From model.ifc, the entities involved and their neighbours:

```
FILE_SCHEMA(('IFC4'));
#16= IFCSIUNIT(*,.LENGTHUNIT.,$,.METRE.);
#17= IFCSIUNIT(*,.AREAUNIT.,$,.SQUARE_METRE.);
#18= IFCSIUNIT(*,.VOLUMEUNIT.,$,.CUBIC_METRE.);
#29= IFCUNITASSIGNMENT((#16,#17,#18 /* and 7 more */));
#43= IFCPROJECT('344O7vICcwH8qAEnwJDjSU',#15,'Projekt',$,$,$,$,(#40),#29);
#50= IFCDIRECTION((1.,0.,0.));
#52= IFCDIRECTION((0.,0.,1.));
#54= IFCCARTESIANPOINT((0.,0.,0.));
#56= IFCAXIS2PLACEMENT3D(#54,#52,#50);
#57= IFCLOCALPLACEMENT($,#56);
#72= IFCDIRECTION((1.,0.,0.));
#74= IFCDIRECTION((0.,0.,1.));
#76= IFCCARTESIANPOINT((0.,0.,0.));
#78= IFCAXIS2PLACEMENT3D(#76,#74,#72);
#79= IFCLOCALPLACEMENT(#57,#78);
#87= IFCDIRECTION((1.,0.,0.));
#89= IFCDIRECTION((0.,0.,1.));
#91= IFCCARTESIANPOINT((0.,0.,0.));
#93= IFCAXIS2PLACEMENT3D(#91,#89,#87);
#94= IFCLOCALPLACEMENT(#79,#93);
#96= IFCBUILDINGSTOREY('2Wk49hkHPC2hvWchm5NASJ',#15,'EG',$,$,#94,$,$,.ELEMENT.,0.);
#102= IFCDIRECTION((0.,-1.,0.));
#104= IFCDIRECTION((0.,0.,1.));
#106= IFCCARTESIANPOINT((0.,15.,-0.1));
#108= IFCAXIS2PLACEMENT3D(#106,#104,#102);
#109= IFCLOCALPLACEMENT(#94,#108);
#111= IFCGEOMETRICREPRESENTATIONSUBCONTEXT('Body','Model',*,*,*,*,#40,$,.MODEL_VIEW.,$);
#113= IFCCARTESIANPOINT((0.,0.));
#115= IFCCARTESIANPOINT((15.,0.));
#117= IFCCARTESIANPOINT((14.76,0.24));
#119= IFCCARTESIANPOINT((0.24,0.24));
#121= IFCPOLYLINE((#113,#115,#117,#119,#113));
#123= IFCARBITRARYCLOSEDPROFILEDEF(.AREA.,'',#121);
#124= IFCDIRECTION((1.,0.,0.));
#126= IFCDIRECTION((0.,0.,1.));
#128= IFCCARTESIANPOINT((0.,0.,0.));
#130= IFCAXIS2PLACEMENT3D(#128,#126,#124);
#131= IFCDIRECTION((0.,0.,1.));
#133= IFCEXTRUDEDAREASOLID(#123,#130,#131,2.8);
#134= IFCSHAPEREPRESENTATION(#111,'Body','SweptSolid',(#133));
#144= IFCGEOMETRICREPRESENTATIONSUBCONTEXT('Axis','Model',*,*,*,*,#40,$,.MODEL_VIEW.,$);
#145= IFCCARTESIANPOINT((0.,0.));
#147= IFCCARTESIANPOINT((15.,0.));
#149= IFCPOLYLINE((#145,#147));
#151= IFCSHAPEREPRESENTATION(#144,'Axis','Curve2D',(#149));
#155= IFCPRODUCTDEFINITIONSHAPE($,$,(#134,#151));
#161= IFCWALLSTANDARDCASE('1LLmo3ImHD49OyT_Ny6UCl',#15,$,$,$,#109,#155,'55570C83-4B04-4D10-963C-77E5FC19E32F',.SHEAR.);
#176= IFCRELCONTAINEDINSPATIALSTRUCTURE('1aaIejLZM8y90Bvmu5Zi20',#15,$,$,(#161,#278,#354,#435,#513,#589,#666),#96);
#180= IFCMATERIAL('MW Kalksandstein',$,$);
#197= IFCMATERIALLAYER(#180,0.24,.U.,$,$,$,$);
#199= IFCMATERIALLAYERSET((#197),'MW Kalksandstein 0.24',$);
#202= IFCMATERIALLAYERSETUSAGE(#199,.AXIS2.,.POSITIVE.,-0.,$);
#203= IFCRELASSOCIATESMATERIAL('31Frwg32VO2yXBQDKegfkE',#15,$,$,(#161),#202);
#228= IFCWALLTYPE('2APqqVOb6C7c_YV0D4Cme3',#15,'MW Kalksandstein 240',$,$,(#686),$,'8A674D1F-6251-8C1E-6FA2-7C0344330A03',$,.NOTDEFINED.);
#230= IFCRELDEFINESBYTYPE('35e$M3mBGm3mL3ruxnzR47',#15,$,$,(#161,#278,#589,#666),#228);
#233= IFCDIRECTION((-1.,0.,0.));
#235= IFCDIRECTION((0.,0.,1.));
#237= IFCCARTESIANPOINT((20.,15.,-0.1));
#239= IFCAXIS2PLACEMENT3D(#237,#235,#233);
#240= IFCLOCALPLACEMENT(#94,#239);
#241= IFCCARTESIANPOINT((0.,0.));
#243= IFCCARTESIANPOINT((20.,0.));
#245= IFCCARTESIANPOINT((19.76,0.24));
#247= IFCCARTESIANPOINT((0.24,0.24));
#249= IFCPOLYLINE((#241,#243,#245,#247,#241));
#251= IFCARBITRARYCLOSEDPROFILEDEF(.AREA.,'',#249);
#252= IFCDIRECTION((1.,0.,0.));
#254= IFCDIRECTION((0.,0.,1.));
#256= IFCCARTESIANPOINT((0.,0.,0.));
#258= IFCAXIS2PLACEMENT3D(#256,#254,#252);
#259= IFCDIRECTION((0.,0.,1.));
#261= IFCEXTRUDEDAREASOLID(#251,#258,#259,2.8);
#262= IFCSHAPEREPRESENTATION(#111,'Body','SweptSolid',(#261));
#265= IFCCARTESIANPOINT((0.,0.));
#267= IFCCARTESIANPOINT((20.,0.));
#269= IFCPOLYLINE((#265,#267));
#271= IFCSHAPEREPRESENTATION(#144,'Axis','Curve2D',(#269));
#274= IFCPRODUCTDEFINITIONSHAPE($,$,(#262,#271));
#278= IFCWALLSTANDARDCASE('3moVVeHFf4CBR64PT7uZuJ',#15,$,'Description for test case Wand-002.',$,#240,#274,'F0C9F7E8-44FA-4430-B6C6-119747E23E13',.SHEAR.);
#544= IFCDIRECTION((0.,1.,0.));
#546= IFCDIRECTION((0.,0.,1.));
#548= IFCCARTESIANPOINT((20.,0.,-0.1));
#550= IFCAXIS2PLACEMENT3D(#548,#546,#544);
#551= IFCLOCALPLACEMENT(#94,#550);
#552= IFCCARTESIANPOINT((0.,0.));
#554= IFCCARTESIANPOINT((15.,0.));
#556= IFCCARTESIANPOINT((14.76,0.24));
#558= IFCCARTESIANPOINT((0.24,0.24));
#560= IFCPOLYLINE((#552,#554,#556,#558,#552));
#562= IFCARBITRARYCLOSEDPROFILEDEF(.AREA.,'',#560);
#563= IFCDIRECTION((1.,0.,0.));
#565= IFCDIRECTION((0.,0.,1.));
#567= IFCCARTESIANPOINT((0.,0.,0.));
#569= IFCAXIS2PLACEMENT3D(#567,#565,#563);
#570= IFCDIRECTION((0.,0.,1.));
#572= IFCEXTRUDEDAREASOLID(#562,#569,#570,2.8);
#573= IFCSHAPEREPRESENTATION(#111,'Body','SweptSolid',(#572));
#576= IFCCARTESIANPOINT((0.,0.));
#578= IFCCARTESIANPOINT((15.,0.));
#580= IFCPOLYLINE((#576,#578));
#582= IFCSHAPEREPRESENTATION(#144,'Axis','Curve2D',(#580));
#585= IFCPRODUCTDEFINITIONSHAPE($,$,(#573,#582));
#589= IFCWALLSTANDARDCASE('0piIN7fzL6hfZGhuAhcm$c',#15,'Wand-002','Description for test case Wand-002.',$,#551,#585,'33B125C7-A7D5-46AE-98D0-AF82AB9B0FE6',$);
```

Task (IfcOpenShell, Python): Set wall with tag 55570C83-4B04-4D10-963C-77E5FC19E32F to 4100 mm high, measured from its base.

```python
import ifcopenshell
import ifcopenshell.geom
import ifcopenshell.util.representation
import ifcopenshell.util.shape

model = ifcopenshell.open("model.ifc")
settings = ifcopenshell.geom.settings()


def volume(element):
    """Net volume in cubic metres, openings subtracted."""
    shape = ifcopenshell.geom.create_shape(settings, element)
    return ifcopenshell.util.shape.get_volume(shape.geometry)


wall = model.by_guid("1LLmo3ImHD49OyT_Ny6UCl")
before = volume(wall)

body = ifcopenshell.util.representation.get_representation(wall, "Model", "Body")
solid = body.Items[0]
old_height = solid.Depth
solid.Depth = 4.1
after = volume(wall)

print(f"height {old_height:g} -> {solid.Depth:g}, volume {before:.3f} -> {after:.3f} m3")

model.write("model_v2.ifc")
```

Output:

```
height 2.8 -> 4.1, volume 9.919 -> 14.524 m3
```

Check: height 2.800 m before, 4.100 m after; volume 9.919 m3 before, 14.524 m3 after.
